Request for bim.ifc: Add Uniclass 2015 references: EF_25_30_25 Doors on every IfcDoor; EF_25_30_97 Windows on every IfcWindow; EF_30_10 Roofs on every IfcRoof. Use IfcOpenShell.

First a look at what the model holds.

```python
import ifcopenshell

model = ifcopenshell.open("bim.ifc")
print(model.schema)
print("classifications:", [c.Name for c in model.by_type("IfcClassification")])
for ifc_class in ("IfcDoor", "IfcRoof", "IfcStair", "IfcWall", "IfcWindow"):
    print(ifc_class, len(model.by_type(ifc_class)))
```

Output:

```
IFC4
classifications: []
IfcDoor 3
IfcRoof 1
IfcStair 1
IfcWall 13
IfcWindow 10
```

```python
import ifcopenshell
import ifcopenshell.api.classification

model = ifcopenshell.open("bim.ifc")

system = ifcopenshell.api.classification.add_classification(model, classification="Uniclass 2015")

codes = {
    "IfcDoor": ("EF_25_30_25", "Doors"),
    "IfcWindow": ("EF_25_30_97", "Windows"),
    "IfcRoof": ("EF_30_10", "Roofs"),
}
for ifc_class, (code, name) in codes.items():
    products = model.by_type(ifc_class)
    ifcopenshell.api.classification.add_reference(
        model, products=products, classification=system, identification=code, name=name
    )
    print(code, len(products))

model.write("bim_edited.ifc")
```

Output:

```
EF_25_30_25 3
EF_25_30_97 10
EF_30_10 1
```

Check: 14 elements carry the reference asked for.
